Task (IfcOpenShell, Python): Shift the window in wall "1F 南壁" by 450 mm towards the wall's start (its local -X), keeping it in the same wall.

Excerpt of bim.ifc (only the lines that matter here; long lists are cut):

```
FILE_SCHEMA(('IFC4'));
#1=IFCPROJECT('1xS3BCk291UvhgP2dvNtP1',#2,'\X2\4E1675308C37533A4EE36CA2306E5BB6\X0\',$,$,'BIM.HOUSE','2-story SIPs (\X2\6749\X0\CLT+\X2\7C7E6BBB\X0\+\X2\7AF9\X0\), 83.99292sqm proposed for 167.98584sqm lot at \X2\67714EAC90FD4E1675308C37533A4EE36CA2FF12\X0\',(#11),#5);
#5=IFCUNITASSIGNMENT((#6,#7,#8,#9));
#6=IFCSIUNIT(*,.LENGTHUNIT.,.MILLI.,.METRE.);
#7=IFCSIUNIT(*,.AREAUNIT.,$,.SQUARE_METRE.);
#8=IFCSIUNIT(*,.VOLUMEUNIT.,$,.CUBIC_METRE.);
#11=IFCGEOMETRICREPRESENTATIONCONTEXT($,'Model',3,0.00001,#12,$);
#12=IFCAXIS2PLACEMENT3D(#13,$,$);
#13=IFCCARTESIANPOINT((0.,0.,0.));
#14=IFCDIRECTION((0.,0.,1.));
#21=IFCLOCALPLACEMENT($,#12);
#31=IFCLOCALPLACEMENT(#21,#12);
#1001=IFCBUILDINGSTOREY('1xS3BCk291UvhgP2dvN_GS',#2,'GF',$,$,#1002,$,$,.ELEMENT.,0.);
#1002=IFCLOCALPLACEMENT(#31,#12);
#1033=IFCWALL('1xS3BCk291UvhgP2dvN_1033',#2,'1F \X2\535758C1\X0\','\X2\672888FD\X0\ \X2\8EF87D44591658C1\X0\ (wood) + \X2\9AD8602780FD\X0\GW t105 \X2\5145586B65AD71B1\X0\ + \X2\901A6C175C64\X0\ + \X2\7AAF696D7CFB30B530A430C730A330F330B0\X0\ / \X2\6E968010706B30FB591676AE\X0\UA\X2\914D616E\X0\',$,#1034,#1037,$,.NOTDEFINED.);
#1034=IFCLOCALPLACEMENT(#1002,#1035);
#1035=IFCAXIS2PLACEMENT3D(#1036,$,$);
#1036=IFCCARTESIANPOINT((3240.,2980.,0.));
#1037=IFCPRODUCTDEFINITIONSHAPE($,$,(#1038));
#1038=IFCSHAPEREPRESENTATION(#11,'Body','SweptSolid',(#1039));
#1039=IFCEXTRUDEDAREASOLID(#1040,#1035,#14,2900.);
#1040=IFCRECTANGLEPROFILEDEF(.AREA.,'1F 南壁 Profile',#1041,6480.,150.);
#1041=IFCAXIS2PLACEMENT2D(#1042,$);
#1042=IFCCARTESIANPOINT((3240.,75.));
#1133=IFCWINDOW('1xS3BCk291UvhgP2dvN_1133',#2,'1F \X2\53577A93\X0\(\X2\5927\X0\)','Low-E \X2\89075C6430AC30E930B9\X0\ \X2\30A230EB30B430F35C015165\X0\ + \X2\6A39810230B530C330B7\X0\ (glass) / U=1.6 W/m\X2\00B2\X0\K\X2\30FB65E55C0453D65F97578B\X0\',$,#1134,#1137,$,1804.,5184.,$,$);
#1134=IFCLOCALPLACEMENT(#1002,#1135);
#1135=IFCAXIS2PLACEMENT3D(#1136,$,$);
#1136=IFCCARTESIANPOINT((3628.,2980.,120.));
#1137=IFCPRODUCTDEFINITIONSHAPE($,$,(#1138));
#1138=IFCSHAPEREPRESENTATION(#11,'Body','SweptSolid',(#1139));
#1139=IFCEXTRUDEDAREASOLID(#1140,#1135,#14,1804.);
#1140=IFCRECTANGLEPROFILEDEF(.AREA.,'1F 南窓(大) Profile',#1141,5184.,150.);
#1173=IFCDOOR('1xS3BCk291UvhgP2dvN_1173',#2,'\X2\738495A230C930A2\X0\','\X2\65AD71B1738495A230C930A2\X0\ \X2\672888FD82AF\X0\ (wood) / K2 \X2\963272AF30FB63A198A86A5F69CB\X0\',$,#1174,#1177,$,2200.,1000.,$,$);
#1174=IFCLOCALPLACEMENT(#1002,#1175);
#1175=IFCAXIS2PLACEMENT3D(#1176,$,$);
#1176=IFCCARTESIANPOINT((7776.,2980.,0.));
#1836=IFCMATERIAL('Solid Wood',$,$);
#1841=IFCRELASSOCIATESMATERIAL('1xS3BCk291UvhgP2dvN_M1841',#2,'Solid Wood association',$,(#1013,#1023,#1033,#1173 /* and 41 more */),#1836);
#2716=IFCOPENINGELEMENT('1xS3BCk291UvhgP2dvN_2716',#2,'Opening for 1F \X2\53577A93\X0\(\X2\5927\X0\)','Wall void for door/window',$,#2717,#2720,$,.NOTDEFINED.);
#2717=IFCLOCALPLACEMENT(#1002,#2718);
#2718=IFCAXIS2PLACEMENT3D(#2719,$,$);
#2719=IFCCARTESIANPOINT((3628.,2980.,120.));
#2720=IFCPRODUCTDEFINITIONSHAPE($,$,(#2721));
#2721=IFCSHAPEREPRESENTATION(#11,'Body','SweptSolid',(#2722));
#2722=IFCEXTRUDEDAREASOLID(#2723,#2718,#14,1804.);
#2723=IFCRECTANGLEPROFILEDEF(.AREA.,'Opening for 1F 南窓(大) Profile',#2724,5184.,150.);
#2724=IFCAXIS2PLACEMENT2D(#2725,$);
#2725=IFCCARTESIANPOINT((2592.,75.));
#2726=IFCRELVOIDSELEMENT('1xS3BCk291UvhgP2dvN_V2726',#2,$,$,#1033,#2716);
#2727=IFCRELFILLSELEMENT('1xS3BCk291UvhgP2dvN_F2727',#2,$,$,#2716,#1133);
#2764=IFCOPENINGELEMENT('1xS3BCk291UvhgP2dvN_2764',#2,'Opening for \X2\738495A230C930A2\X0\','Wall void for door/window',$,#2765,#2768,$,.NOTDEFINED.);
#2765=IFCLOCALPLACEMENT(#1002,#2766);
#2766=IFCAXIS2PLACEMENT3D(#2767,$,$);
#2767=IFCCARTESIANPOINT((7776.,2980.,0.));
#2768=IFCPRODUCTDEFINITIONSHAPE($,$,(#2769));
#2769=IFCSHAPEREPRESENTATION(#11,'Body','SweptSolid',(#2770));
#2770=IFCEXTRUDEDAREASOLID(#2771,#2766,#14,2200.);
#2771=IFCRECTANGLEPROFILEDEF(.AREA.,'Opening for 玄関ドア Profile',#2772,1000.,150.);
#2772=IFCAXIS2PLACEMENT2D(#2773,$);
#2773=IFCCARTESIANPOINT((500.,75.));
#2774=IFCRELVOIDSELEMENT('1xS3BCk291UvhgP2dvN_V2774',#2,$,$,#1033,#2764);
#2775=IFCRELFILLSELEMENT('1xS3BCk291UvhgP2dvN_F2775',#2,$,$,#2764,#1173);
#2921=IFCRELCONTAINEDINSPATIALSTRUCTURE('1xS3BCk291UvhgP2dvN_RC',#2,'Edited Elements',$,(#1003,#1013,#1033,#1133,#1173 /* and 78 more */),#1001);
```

```python
import ifcopenshell
import ifcopenshell.api.geometry
import ifcopenshell.util.placement

model = ifcopenshell.open("bim.ifc")

window = model.by_id(1133)
opening = window.FillsVoids[0].RelatingOpeningElement
wall = opening.VoidsElements[0].RelatingBuildingElement

wall_matrix = ifcopenshell.util.placement.get_local_placement(wall.ObjectPlacement)
shift = wall_matrix[:3, 0] * -450.0
before = ifcopenshell.util.placement.get_local_placement(window.ObjectPlacement)[:3, 3].copy()

# The window is not placed relative to its opening, so move both.
for product in (opening, window):
    matrix = ifcopenshell.util.placement.get_local_placement(product.ObjectPlacement)
    matrix[:3, 3] += shift
    ifcopenshell.api.geometry.edit_object_placement(model, product=product, matrix=matrix, is_si=False)

after = ifcopenshell.util.placement.get_local_placement(window.ObjectPlacement)[:3, 3]
print("window moved by", (after - before).round(3) + 0.0)

model.write("bim-out.ifc")
```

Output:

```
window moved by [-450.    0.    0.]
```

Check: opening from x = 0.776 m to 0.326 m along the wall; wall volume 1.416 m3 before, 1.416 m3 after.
